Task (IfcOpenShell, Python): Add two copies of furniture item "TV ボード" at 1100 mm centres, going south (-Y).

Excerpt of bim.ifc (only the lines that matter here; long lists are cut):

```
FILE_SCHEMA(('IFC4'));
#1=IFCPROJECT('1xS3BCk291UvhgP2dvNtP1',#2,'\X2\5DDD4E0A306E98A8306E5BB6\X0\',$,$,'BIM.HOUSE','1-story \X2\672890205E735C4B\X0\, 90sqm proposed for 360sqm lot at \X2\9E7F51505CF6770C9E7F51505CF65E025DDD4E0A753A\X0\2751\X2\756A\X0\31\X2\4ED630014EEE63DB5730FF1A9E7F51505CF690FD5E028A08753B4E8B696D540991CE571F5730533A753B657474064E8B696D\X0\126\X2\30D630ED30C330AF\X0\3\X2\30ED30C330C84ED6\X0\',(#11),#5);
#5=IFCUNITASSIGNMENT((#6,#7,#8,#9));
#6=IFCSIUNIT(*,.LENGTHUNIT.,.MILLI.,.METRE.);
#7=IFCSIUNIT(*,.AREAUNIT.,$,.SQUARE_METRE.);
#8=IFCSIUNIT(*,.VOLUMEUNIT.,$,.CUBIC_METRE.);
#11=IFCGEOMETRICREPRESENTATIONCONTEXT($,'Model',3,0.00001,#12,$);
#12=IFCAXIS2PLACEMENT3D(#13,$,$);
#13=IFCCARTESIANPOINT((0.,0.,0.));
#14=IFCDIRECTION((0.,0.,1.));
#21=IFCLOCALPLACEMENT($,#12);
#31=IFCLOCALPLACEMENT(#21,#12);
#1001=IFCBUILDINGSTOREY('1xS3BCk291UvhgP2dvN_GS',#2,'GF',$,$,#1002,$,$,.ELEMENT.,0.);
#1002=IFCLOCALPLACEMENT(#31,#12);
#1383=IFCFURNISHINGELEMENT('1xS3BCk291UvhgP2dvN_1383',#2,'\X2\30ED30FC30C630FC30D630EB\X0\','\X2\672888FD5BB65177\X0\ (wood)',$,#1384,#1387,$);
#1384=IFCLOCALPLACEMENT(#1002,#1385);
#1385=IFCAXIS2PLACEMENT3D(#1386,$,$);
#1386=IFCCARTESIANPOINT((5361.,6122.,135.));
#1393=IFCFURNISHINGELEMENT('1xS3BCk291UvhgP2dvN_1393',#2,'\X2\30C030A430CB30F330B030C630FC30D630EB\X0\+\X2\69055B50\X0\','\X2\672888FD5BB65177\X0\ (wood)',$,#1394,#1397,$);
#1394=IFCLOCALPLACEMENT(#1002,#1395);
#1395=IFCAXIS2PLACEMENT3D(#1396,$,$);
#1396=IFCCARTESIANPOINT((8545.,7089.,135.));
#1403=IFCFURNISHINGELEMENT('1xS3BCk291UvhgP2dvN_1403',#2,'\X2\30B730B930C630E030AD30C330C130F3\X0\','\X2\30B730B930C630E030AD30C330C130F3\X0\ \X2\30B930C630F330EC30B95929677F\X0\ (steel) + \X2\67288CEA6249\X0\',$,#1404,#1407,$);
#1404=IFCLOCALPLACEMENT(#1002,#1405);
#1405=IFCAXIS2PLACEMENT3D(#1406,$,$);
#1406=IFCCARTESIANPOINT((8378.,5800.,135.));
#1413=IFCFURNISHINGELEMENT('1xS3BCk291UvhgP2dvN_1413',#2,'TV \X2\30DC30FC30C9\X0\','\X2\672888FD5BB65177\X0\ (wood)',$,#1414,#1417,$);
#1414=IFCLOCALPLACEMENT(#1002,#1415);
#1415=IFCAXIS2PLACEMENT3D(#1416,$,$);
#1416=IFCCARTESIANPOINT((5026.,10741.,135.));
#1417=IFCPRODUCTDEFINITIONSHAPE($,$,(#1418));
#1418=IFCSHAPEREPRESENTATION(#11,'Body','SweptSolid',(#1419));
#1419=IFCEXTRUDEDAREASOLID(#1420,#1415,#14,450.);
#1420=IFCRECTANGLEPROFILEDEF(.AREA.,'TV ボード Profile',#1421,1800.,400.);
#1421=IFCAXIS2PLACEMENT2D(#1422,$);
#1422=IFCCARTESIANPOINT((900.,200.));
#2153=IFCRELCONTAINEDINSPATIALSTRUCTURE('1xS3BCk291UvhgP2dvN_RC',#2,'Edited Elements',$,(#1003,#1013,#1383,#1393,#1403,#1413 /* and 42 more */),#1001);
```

```python
import numpy as np
import ifcopenshell
import ifcopenshell.api.geometry
import ifcopenshell.api.root
import ifcopenshell.util.element
import ifcopenshell.util.placement
import ifcopenshell.util.unit

model = ifcopenshell.open("bim.ifc")
unit_scale = ifcopenshell.util.unit.calculate_unit_scale(model)


def reuse_history(source, copy):
    """copy_class also copies each property set's owner history, people and application; keep the originals."""
    for rel in copy.IsDefinedBy:
        if rel.is_a("IfcRelDefinesByProperties") and (history := rel.RelatingPropertyDefinition.OwnerHistory):
            rel.RelatingPropertyDefinition.OwnerHistory = source.OwnerHistory
            ifcopenshell.util.element.remove_deep2(model, history)


source = model.by_guid("1xS3BCk291UvhgP2dvN_1413")
base = ifcopenshell.util.placement.get_local_placement(source.ObjectPlacement)
step = np.array([0.0, -1.0, 0.0]) * 1.1 / unit_scale

for i in range(1, 3):
    copy = ifcopenshell.api.root.copy_class(model, product=source)
    copy.Representation = ifcopenshell.util.element.copy_deep(
        model, source.Representation, exclude=["IfcGeometricRepresentationContext", "IfcRepresentationMap"]
    )
    reuse_history(source, copy)
    matrix = base.copy()
    matrix[:3, 3] += i * step
    print("added at", matrix[:3, 3].round(3) + 0.0)
    ifcopenshell.api.geometry.edit_object_placement(model, product=copy, matrix=matrix, is_si=False)

model.write("bim-out.ifc")
```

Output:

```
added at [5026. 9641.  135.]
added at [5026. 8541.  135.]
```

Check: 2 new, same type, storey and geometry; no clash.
